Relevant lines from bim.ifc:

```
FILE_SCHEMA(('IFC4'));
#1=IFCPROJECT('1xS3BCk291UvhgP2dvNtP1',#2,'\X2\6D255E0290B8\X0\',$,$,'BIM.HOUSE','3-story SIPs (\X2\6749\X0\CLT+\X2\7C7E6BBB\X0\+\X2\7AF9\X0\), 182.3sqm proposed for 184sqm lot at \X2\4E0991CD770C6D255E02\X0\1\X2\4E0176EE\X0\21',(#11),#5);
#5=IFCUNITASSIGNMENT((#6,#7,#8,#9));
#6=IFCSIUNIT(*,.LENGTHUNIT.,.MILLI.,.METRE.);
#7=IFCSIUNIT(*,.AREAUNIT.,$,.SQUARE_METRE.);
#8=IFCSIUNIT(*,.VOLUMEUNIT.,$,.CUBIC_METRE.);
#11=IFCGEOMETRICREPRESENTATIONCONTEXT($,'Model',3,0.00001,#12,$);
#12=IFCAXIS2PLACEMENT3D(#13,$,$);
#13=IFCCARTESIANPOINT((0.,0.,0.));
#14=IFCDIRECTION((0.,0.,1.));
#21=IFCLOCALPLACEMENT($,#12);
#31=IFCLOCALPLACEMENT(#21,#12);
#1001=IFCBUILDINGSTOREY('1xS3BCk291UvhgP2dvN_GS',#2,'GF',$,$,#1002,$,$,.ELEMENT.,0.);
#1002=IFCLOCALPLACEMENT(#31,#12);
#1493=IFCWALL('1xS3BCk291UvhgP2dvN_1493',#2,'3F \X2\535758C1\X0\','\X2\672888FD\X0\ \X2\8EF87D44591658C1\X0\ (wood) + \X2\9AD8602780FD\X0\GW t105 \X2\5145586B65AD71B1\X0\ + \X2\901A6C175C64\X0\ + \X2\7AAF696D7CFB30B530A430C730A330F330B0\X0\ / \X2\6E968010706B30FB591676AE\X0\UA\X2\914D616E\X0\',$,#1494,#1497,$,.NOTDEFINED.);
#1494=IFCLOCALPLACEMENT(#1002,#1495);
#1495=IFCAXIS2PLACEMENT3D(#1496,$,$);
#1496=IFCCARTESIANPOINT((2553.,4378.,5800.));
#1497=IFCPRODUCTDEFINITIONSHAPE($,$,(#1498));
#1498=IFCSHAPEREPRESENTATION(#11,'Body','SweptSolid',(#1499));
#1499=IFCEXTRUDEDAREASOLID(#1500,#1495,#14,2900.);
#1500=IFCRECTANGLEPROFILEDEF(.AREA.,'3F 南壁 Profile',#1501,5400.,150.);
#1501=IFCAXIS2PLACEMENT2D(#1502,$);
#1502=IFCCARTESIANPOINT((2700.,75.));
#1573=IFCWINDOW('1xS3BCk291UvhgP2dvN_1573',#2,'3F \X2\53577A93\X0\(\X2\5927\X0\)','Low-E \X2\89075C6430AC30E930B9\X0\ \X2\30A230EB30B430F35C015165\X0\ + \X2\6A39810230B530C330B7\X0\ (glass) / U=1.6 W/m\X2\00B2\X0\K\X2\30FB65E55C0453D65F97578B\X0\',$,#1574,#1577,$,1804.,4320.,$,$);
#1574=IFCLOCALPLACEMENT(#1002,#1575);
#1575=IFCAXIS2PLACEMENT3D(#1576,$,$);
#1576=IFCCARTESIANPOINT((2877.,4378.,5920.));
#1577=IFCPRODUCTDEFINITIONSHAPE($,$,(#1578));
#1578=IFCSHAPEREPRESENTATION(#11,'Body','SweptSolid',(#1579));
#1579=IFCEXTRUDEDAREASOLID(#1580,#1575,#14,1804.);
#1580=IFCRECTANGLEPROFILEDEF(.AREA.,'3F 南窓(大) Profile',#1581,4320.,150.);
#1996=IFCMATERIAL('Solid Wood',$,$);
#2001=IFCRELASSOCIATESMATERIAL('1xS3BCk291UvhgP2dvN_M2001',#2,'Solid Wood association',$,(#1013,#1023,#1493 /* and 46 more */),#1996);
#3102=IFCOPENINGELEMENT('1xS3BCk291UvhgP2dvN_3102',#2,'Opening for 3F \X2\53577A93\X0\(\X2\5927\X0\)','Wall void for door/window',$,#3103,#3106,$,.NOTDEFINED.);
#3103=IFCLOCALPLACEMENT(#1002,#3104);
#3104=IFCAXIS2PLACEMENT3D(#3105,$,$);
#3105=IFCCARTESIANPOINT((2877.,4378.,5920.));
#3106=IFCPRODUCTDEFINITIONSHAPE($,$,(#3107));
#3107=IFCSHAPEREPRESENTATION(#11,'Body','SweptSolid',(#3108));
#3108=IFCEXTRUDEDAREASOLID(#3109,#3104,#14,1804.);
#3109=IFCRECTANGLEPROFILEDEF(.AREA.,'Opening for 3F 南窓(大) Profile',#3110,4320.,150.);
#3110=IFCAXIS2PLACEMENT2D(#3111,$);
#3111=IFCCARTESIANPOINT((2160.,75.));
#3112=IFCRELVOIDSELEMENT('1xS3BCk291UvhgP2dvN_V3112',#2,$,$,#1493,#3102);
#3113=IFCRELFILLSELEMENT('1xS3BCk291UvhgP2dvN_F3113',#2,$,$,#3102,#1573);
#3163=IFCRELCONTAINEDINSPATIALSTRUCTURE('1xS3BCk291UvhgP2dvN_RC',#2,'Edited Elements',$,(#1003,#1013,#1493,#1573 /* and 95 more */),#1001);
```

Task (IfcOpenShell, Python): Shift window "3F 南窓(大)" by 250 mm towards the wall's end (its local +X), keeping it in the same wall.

```python
import ifcopenshell
import ifcopenshell.api.geometry
import ifcopenshell.util.placement
import ifcopenshell.util.unit

model = ifcopenshell.open("bim.ifc")
unit_scale = ifcopenshell.util.unit.calculate_unit_scale(model)

window = model.by_guid("1xS3BCk291UvhgP2dvN_1573")
opening = window.FillsVoids[0].RelatingOpeningElement
wall = opening.VoidsElements[0].RelatingBuildingElement

wall_matrix = ifcopenshell.util.placement.get_local_placement(wall.ObjectPlacement)
shift = wall_matrix[:3, 0] * 0.25 / unit_scale
before = ifcopenshell.util.placement.get_local_placement(window.ObjectPlacement)[:3, 3].copy()

# The window is not placed relative to its opening, so move both.
for product in (opening, window):
    matrix = ifcopenshell.util.placement.get_local_placement(product.ObjectPlacement)
    matrix[:3, 3] += shift
    ifcopenshell.api.geometry.edit_object_placement(model, product=product, matrix=matrix, is_si=False)

after = ifcopenshell.util.placement.get_local_placement(window.ObjectPlacement)[:3, 3]
print("window moved by", (after - before).round(3) + 0.0)

model.write("bim-out.ifc")
```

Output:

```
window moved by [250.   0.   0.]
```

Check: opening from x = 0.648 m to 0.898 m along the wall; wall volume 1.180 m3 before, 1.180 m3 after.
